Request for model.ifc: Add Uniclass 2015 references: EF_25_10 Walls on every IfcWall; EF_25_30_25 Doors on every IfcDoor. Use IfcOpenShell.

First a look at what the model holds.

```python
import ifcopenshell

model = ifcopenshell.open("model.ifc")
print(model.schema)
print("classifications:", [c.Name for c in model.by_type("IfcClassification")])
for ifc_class in ("IfcDoor", "IfcRoof", "IfcStair", "IfcWall", "IfcWindow"):
    print(ifc_class, len(model.by_type(ifc_class)))
```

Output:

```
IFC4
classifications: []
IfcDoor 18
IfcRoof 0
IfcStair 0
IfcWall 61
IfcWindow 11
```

```python
import ifcopenshell
import ifcopenshell.api.classification

model = ifcopenshell.open("model.ifc")

system = ifcopenshell.api.classification.add_classification(model, classification="Uniclass 2015")

codes = {
    "IfcWall": ("EF_25_10", "Walls"),
    "IfcDoor": ("EF_25_30_25", "Doors"),
}
for ifc_class, (code, name) in codes.items():
    products = model.by_type(ifc_class)
    ifcopenshell.api.classification.add_reference(
        model, products=products, classification=system, identification=code, name=name
    )
    print(code, len(products))

model.write("model_updated.ifc")
```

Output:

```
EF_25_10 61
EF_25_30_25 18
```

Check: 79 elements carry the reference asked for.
